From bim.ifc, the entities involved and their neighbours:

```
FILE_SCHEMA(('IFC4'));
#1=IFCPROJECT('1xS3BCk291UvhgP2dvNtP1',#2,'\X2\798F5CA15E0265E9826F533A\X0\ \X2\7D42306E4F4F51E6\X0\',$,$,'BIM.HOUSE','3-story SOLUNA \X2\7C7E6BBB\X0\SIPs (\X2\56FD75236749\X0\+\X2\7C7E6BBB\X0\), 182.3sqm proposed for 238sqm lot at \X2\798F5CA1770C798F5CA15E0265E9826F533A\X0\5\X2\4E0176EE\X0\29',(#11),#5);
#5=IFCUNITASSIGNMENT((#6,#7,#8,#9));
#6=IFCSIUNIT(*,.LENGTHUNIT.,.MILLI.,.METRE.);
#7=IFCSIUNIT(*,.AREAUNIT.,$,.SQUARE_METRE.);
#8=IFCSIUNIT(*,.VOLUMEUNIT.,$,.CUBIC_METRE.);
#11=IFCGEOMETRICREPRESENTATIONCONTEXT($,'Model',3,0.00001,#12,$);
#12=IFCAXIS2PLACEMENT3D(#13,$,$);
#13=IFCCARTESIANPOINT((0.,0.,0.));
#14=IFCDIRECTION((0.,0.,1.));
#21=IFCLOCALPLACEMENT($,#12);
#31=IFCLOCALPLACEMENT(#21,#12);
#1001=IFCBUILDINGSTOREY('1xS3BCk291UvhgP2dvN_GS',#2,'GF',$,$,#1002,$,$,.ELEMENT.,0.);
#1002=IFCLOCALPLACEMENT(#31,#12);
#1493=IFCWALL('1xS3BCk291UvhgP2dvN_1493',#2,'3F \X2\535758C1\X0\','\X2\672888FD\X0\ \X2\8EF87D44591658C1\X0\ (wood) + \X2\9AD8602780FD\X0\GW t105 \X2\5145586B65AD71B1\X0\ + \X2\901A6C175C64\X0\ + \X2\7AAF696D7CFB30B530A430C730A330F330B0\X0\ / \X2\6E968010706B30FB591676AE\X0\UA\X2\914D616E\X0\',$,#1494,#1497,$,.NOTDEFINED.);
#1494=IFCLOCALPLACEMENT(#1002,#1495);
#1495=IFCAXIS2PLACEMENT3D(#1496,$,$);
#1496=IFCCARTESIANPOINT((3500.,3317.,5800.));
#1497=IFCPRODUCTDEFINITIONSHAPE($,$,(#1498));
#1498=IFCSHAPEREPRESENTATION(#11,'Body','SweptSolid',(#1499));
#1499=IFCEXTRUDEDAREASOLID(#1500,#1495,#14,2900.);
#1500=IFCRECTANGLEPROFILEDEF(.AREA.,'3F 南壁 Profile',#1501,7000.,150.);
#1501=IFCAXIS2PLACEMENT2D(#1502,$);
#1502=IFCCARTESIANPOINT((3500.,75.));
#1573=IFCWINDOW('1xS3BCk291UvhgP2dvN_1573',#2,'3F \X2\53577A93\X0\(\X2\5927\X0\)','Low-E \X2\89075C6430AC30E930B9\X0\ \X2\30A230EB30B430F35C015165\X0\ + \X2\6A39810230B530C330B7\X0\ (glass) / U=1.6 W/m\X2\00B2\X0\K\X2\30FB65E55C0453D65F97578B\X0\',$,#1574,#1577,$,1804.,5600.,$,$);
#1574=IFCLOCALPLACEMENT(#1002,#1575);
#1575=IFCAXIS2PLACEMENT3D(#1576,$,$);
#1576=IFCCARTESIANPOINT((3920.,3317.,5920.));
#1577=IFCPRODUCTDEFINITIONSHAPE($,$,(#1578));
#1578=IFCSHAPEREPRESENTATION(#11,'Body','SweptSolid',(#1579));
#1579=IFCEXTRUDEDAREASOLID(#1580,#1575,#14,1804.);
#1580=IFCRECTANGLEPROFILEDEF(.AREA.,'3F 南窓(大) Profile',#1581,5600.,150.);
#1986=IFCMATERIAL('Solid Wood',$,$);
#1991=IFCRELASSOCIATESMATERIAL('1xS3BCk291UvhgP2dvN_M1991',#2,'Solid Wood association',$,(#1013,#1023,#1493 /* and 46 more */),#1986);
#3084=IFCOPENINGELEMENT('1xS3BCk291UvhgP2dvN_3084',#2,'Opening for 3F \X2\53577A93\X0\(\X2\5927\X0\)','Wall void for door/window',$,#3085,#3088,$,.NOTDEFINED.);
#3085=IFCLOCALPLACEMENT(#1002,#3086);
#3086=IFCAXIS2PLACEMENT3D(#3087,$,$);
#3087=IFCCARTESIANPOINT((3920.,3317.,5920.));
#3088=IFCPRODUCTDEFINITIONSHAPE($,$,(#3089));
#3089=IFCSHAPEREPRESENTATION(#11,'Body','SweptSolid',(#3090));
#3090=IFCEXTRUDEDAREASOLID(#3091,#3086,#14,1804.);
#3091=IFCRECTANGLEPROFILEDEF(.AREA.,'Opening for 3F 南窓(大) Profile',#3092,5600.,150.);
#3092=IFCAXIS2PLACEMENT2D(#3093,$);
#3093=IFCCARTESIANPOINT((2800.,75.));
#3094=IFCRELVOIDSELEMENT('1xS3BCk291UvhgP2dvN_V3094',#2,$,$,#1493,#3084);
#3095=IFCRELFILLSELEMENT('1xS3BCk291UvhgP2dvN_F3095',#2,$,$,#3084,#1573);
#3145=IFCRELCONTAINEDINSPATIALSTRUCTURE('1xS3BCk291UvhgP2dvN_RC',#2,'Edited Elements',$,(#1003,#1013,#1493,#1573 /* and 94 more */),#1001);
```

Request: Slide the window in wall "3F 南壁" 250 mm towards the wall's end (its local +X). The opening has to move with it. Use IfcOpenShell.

```python
import ifcopenshell
import ifcopenshell.api.geometry
import ifcopenshell.util.placement

model = ifcopenshell.open("bim.ifc")

window = model.by_guid("1xS3BCk291UvhgP2dvN_1573")
opening = window.FillsVoids[0].RelatingOpeningElement
wall = opening.VoidsElements[0].RelatingBuildingElement

wall_matrix = ifcopenshell.util.placement.get_local_placement(wall.ObjectPlacement)
shift = wall_matrix[:3, 0] * 250.0
before = ifcopenshell.util.placement.get_local_placement(window.ObjectPlacement)[:3, 3].copy()

# The window is not placed relative to its opening, so move both.
for product in (opening, window):
    matrix = ifcopenshell.util.placement.get_local_placement(product.ObjectPlacement)
    matrix[:3, 3] += shift
    ifcopenshell.api.geometry.edit_object_placement(model, product=product, matrix=matrix, is_si=False)

after = ifcopenshell.util.placement.get_local_placement(window.ObjectPlacement)[:3, 3]
print("window moved by", (after - before).round(3) + 0.0)

model.write("bim_updated.ifc")
```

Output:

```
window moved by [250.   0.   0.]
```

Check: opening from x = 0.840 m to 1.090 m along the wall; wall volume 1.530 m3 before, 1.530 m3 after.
